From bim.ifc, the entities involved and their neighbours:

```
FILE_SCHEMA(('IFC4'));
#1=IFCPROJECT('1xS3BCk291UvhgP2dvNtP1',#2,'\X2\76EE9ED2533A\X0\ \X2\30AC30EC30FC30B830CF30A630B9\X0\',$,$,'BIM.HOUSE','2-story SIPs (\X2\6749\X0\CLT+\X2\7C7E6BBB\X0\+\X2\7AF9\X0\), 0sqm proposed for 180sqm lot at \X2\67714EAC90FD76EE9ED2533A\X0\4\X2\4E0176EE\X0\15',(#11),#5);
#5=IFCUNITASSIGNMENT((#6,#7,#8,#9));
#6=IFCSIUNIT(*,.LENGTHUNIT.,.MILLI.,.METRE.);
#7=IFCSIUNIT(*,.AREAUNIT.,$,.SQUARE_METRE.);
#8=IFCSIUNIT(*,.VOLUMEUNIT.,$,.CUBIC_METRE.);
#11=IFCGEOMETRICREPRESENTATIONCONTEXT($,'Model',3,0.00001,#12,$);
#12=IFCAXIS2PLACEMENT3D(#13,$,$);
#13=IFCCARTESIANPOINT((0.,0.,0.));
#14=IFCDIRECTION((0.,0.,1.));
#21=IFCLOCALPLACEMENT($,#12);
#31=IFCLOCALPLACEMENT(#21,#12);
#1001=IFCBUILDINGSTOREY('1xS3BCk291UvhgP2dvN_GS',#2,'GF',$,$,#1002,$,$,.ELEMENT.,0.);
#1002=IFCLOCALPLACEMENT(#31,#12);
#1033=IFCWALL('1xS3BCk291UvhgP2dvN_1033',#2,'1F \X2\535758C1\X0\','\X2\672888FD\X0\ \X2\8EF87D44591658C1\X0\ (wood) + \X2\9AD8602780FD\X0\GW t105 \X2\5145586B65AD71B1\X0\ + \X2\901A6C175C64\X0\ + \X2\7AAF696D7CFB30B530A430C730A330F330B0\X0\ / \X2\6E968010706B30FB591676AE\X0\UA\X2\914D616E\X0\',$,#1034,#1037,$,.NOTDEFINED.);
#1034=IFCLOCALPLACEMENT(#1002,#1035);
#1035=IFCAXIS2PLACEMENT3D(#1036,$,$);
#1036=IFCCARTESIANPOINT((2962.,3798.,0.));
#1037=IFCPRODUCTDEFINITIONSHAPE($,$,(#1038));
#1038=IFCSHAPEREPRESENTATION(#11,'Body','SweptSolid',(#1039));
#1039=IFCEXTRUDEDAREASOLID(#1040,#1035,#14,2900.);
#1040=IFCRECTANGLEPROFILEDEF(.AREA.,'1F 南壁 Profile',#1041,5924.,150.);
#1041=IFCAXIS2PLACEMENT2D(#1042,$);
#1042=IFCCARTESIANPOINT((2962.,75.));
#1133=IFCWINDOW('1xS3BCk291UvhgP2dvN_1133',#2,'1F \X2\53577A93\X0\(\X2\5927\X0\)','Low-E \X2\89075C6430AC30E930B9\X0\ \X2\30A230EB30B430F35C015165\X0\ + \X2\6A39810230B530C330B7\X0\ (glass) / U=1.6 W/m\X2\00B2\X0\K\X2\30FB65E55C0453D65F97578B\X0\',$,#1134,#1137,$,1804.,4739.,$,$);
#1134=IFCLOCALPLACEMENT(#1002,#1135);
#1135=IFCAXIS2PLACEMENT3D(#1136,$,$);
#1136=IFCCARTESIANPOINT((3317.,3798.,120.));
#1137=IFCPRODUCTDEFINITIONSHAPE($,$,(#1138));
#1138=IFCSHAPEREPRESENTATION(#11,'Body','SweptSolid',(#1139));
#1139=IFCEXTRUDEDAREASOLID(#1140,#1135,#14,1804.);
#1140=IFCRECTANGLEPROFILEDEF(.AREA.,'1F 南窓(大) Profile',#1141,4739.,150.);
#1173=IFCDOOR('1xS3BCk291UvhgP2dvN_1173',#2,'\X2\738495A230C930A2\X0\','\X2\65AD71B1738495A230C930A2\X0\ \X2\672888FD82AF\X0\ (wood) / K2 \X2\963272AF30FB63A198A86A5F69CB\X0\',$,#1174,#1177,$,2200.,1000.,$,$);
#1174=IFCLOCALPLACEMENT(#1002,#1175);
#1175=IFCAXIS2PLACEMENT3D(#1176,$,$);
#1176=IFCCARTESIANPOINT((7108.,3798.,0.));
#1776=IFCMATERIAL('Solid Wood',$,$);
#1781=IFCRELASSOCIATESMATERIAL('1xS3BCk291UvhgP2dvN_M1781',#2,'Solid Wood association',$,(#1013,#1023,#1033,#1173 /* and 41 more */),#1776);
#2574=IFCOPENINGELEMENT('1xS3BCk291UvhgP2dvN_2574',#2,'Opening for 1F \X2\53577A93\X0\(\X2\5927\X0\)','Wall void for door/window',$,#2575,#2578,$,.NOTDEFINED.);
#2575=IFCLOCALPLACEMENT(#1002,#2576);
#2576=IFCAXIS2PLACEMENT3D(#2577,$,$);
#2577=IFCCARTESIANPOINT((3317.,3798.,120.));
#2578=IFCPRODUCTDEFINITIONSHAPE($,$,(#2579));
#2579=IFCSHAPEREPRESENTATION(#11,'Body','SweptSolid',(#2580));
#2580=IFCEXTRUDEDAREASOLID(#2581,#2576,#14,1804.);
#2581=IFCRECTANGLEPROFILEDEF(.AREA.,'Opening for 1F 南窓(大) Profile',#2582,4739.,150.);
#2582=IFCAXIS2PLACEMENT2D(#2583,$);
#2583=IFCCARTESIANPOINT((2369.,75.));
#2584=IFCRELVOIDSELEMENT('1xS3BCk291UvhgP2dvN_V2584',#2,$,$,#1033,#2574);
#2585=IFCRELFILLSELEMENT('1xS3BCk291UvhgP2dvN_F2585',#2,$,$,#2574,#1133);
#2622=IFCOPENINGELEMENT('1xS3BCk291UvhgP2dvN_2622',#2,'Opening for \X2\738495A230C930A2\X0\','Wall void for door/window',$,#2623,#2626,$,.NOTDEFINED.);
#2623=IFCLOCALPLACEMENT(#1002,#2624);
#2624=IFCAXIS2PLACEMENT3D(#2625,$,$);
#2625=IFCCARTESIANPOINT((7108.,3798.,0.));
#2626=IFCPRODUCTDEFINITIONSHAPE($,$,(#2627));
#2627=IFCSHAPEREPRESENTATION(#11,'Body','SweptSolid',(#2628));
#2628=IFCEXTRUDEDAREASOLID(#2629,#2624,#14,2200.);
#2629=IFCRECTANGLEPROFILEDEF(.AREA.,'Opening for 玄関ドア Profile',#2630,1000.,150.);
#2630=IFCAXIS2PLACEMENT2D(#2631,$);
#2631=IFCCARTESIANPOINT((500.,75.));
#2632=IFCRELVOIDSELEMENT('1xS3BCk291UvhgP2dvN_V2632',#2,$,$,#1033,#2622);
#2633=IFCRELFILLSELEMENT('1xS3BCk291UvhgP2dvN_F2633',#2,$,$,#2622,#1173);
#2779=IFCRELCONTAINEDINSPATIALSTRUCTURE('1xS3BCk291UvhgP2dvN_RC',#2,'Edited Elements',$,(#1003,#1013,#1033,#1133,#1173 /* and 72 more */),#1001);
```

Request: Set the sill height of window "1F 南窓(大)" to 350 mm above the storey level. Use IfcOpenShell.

```python
import numpy as np
import ifcopenshell
import ifcopenshell.api.geometry
import ifcopenshell.geom
import ifcopenshell.util.element
import ifcopenshell.util.placement
import ifcopenshell.util.shape
import ifcopenshell.util.unit

model = ifcopenshell.open("bim.ifc")
unit_scale = ifcopenshell.util.unit.calculate_unit_scale(model)

window = model.by_guid("1xS3BCk291UvhgP2dvN_1133")
opening = window.FillsVoids[0].RelatingOpeningElement
storey = ifcopenshell.util.element.get_container(window, ifc_class="IfcBuildingStorey")
level = ifcopenshell.util.placement.get_local_placement(storey.ObjectPlacement)[2, 3]

# The opening's origin need not be at the sill, so measure its lowest point.
shape = ifcopenshell.geom.create_shape(ifcopenshell.geom.settings(), opening)
bottom = ifcopenshell.util.shape.get_shape_bottom_elevation(shape, shape.geometry) / unit_scale
dz = level + 350.0 - bottom

shift = np.array([0.0, 0.0, dz])
# The window is not placed relative to its opening, so move both.
for product in (opening, window):
    matrix = ifcopenshell.util.placement.get_local_placement(product.ObjectPlacement)
    matrix[:3, 3] += shift
    ifcopenshell.api.geometry.edit_object_placement(model, product=product, matrix=matrix, is_si=False)

print(f"moved by {dz * unit_scale:+.3f} m")

model.write("bim_v2.ifc")
```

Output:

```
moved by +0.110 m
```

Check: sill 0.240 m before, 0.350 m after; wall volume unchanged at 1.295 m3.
